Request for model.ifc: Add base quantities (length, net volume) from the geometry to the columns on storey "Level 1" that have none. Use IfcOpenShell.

First a look at what the model holds.

```python
import ifcopenshell
import ifcopenshell.util.element
import ifcopenshell.util.unit

model = ifcopenshell.open("model.ifc")
print(model.schema)
for unit_type in ("LENGTHUNIT", "AREAUNIT", "VOLUMEUNIT"):
    print(unit_type, ifcopenshell.util.unit.calculate_unit_scale(model, unit_type))
storey = next(s for s in model.by_type("IfcBuildingStorey") if s.Name == "Level 1")
columns = [e for e in ifcopenshell.util.element.get_decomposition(storey) if e.is_a("IfcColumn")]
for e in sorted(columns, key=lambda e: e.id()):
    print(e.id(), e.is_a(), e.Name, list(ifcopenshell.util.element.get_psets(e, qtos_only=True)), sep=" | ")
```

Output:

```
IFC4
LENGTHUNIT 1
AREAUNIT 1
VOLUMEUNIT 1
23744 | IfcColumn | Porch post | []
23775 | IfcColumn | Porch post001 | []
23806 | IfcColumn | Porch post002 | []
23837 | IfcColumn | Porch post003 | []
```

```python
import ifcopenshell
import ifcopenshell.api.pset
import ifcopenshell.geom
import ifcopenshell.util.element
import ifcopenshell.util.shape
import ifcopenshell.util.unit

model = ifcopenshell.open("model.ifc")
unit_scale = ifcopenshell.util.unit.calculate_unit_scale(model)
volume_scale = ifcopenshell.util.unit.calculate_unit_scale(model, "VOLUMEUNIT")
settings = ifcopenshell.geom.settings()

storey = next(s for s in model.by_type("IfcBuildingStorey") if s.Name == "Level 1")
columns = [e for e in ifcopenshell.util.element.get_decomposition(storey) if e.is_a("IfcColumn")]

for e in sorted(columns, key=lambda e: e.id()):
    if ifcopenshell.util.element.get_psets(e, qtos_only=True, should_inherit=False):
        continue
    # Geometry comes back in metres, in the element's own axes.
    shape = ifcopenshell.geom.create_shape(settings, e)
    values = {
        "Length": ifcopenshell.util.shape.get_z(shape.geometry) / unit_scale,
        "NetVolume": ifcopenshell.util.shape.get_volume(shape.geometry) / volume_scale,
    }
    qto = ifcopenshell.api.pset.add_qto(model, product=e, name="Qto_ColumnBaseQuantities")
    ifcopenshell.api.pset.edit_qto(model, qto=qto, properties=values)
    print(e.id(), {k: round(v, 3) for k, v in values.items()})

model.write("model_v2.ifc")
```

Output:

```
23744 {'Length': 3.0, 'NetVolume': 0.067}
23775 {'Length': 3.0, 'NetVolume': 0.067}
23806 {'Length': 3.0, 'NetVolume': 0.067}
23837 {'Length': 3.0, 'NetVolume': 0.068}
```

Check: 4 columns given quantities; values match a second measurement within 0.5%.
